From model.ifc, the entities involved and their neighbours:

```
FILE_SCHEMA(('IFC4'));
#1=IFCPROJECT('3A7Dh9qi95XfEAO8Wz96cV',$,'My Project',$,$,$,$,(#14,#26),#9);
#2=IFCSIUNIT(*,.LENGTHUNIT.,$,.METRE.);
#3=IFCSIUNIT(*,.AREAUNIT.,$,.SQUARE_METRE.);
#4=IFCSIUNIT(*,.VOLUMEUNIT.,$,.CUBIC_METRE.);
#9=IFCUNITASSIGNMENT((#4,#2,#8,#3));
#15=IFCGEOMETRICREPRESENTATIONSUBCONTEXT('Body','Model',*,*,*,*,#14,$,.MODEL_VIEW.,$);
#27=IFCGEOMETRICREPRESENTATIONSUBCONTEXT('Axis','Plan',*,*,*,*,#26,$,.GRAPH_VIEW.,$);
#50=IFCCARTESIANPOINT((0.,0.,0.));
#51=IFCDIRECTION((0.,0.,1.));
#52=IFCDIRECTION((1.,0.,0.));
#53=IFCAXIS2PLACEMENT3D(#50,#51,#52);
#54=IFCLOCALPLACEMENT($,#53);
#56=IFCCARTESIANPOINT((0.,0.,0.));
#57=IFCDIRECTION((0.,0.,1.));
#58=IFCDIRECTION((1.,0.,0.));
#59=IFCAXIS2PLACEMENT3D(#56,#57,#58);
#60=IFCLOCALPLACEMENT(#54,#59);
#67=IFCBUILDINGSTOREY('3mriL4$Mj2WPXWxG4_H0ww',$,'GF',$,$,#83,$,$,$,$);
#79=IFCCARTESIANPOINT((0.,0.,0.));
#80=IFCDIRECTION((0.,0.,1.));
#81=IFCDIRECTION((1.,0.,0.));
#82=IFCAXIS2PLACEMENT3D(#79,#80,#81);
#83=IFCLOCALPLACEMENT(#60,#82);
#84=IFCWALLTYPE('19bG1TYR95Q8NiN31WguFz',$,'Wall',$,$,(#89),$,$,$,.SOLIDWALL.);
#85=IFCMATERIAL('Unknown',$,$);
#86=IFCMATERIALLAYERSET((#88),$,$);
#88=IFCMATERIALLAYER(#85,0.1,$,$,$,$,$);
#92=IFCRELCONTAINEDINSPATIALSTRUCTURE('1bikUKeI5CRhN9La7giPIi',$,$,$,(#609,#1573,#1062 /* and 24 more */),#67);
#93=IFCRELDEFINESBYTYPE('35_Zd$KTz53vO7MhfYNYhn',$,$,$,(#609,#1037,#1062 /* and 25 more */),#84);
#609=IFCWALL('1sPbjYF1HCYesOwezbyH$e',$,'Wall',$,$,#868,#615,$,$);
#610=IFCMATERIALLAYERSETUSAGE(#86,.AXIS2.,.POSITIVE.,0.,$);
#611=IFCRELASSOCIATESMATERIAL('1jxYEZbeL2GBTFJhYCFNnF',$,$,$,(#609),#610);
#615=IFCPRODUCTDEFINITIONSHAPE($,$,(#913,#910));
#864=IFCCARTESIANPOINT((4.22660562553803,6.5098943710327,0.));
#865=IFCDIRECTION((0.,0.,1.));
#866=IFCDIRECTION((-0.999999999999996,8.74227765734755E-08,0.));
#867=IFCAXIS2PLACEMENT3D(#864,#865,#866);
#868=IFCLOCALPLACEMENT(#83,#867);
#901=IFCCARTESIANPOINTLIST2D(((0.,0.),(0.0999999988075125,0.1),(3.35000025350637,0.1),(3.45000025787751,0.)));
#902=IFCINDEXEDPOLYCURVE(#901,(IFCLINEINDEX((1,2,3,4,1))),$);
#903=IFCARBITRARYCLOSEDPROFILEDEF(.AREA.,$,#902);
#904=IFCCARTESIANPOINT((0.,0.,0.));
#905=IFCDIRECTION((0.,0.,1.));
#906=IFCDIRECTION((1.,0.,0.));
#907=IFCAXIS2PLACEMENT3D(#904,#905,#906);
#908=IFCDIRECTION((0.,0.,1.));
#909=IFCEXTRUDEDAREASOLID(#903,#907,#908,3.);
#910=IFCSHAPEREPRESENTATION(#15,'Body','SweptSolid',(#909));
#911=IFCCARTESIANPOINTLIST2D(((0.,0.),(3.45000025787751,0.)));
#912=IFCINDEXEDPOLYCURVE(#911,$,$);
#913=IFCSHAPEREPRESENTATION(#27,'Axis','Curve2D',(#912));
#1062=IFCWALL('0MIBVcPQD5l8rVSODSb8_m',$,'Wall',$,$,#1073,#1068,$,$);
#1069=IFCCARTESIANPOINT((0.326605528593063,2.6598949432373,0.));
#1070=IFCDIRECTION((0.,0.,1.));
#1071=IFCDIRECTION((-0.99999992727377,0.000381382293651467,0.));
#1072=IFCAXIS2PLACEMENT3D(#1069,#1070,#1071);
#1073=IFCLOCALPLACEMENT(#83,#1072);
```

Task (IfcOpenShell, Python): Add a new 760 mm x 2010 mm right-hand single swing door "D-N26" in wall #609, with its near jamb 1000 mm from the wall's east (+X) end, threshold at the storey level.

```python
import numpy as np
import ifcopenshell
import ifcopenshell.api.feature
import ifcopenshell.api.geometry
import ifcopenshell.api.root
import ifcopenshell.api.spatial
import ifcopenshell.geom
import ifcopenshell.util.element
import ifcopenshell.util.placement
import ifcopenshell.util.representation
import ifcopenshell.util.shape
import ifcopenshell.util.unit

model = ifcopenshell.open("model.ifc")
unit_scale = ifcopenshell.util.unit.calculate_unit_scale(model)
settings = ifcopenshell.geom.settings()


def volume(element):
    """Net volume in cubic metres, openings subtracted."""
    shape = ifcopenshell.geom.create_shape(settings, element)
    return ifcopenshell.util.shape.get_volume(shape.geometry)


wall = model.by_id(609)
storey = ifcopenshell.util.element.get_container(wall, ifc_class="IfcBuildingStorey")
context = ifcopenshell.util.representation.get_context(model, "Model", "Body", "MODEL_VIEW")
before = volume(wall)

width, height, from_end, sill = 0.76, 2.01, 1, 0.0  # metres

# The wall runs along its own X axis, and the end named is its -X end.
wall_shape = ifcopenshell.geom.create_shape(settings, wall)
x, y, z = ifcopenshell.util.shape.get_vertices(wall_shape.geometry).T
start = x.min() + from_end
face, thickness = float(y.min()), float(y.max() - y.min())
wall_matrix = ifcopenshell.util.placement.get_local_placement(wall.ObjectPlacement)
level = ifcopenshell.util.placement.get_local_placement(storey.ObjectPlacement)[2, 3]


def in_wall(x, y):
    """Placement at x, y metres in the wall's axes, at sill height."""
    matrix = wall_matrix.copy()
    matrix[:, 3] = wall_matrix @ np.array([x / unit_scale, y / unit_scale, 0.0, 1.0])
    matrix[2, 3] = level + sill / unit_scale
    return matrix


# Opening: a box that overshoots both wall faces by 50 mm.
opening = ifcopenshell.api.root.create_entity(model, ifc_class="IfcOpeningElement", predefined_type="OPENING")
box = ifcopenshell.api.geometry.add_wall_representation(
    model, context=context, length=width, height=height, thickness=thickness + 0.1
)
ifcopenshell.api.geometry.assign_representation(model, product=opening, representation=box)
ifcopenshell.api.geometry.edit_object_placement(model, product=opening, matrix=in_wall(start, face - 0.05), is_si=False)
ifcopenshell.api.feature.add_feature(model, feature=opening, element=wall)

door = ifcopenshell.api.root.create_entity(model, ifc_class="IfcDoor", name="D-N26", predefined_type="DOOR")
door.OverallWidth, door.OverallHeight = width / unit_scale, height / unit_scale
door.OperationType = "SINGLE_SWING_RIGHT"
body = ifcopenshell.api.geometry.add_door_representation(
    model,
    context=context,
    overall_width=door.OverallWidth,
    overall_height=door.OverallHeight,
    operation_type="SINGLE_SWING_RIGHT",
    lining_properties={"LiningDepth": thickness / unit_scale, "ThresholdDepth": thickness / unit_scale},
)
ifcopenshell.api.geometry.assign_representation(model, product=door, representation=body)
ifcopenshell.api.spatial.assign_container(model, products=[door], relating_structure=storey)
ifcopenshell.api.feature.add_filling(model, opening=opening, element=door)

# The lining spans the wall, so the door starts at the wall face.
ifcopenshell.api.geometry.edit_object_placement(model, product=door, matrix=in_wall(start, face), is_si=False)

after = volume(wall)

print(f"wall volume {before:.3f} -> {after:.3f} m3")

model.write("model_updated.ifc")
```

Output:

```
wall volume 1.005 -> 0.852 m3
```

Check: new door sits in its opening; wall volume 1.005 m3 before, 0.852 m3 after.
